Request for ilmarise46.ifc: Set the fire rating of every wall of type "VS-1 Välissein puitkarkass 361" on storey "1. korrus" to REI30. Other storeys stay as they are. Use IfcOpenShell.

First a look at what the model holds.

```python
import ifcopenshell
import ifcopenshell.util.element

model = ifcopenshell.open("ilmarise46.ifc")
print(model.schema)
storey = next(s for s in model.by_type("IfcBuildingStorey") if s.Name == "1. korrus")
walls = [e for e in ifcopenshell.util.element.get_decomposition(storey) if e.is_a("IfcWall")]
seen = {}
for e in walls:
    element_type = ifcopenshell.util.element.get_type(e)
    key = (element_type.Name if element_type != e and element_type else None, ifcopenshell.util.element.get_pset(e, "Pset_WallCommon", "FireRating"))
    seen[key] = seen.get(key, 0) + 1
for (name, value), count in sorted(seen.items(), key=str):
    print(count, "x", name, "|", value)
```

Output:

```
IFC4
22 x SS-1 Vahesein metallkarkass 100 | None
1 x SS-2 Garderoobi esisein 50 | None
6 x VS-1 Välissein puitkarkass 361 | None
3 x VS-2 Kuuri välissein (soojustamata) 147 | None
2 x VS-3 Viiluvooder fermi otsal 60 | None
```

```python
import ifcopenshell
import ifcopenshell.api.pset
import ifcopenshell.util.element

model = ifcopenshell.open("ilmarise46.ifc")

storey = next(s for s in model.by_type("IfcBuildingStorey") if s.Name == "1. korrus")
walls = [e for e in ifcopenshell.util.element.get_decomposition(storey) if e.is_a("IfcWall")]

count = 0
for e in walls:
    element_type = ifcopenshell.util.element.get_type(e)
    if element_type in (None, e) or element_type.Name != "VS-1 Välissein puitkarkass 361":
        continue
    # add_pset returns the element's existing set when there is one.
    pset = ifcopenshell.api.pset.add_pset(model, product=e, name="Pset_WallCommon")
    ifcopenshell.api.pset.edit_pset(model, pset=pset, properties={"FireRating": "REI30"})
    count += 1

print(count, "walls updated")

model.write("ilmarise46_edited.ifc")
```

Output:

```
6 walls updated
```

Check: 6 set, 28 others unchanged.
